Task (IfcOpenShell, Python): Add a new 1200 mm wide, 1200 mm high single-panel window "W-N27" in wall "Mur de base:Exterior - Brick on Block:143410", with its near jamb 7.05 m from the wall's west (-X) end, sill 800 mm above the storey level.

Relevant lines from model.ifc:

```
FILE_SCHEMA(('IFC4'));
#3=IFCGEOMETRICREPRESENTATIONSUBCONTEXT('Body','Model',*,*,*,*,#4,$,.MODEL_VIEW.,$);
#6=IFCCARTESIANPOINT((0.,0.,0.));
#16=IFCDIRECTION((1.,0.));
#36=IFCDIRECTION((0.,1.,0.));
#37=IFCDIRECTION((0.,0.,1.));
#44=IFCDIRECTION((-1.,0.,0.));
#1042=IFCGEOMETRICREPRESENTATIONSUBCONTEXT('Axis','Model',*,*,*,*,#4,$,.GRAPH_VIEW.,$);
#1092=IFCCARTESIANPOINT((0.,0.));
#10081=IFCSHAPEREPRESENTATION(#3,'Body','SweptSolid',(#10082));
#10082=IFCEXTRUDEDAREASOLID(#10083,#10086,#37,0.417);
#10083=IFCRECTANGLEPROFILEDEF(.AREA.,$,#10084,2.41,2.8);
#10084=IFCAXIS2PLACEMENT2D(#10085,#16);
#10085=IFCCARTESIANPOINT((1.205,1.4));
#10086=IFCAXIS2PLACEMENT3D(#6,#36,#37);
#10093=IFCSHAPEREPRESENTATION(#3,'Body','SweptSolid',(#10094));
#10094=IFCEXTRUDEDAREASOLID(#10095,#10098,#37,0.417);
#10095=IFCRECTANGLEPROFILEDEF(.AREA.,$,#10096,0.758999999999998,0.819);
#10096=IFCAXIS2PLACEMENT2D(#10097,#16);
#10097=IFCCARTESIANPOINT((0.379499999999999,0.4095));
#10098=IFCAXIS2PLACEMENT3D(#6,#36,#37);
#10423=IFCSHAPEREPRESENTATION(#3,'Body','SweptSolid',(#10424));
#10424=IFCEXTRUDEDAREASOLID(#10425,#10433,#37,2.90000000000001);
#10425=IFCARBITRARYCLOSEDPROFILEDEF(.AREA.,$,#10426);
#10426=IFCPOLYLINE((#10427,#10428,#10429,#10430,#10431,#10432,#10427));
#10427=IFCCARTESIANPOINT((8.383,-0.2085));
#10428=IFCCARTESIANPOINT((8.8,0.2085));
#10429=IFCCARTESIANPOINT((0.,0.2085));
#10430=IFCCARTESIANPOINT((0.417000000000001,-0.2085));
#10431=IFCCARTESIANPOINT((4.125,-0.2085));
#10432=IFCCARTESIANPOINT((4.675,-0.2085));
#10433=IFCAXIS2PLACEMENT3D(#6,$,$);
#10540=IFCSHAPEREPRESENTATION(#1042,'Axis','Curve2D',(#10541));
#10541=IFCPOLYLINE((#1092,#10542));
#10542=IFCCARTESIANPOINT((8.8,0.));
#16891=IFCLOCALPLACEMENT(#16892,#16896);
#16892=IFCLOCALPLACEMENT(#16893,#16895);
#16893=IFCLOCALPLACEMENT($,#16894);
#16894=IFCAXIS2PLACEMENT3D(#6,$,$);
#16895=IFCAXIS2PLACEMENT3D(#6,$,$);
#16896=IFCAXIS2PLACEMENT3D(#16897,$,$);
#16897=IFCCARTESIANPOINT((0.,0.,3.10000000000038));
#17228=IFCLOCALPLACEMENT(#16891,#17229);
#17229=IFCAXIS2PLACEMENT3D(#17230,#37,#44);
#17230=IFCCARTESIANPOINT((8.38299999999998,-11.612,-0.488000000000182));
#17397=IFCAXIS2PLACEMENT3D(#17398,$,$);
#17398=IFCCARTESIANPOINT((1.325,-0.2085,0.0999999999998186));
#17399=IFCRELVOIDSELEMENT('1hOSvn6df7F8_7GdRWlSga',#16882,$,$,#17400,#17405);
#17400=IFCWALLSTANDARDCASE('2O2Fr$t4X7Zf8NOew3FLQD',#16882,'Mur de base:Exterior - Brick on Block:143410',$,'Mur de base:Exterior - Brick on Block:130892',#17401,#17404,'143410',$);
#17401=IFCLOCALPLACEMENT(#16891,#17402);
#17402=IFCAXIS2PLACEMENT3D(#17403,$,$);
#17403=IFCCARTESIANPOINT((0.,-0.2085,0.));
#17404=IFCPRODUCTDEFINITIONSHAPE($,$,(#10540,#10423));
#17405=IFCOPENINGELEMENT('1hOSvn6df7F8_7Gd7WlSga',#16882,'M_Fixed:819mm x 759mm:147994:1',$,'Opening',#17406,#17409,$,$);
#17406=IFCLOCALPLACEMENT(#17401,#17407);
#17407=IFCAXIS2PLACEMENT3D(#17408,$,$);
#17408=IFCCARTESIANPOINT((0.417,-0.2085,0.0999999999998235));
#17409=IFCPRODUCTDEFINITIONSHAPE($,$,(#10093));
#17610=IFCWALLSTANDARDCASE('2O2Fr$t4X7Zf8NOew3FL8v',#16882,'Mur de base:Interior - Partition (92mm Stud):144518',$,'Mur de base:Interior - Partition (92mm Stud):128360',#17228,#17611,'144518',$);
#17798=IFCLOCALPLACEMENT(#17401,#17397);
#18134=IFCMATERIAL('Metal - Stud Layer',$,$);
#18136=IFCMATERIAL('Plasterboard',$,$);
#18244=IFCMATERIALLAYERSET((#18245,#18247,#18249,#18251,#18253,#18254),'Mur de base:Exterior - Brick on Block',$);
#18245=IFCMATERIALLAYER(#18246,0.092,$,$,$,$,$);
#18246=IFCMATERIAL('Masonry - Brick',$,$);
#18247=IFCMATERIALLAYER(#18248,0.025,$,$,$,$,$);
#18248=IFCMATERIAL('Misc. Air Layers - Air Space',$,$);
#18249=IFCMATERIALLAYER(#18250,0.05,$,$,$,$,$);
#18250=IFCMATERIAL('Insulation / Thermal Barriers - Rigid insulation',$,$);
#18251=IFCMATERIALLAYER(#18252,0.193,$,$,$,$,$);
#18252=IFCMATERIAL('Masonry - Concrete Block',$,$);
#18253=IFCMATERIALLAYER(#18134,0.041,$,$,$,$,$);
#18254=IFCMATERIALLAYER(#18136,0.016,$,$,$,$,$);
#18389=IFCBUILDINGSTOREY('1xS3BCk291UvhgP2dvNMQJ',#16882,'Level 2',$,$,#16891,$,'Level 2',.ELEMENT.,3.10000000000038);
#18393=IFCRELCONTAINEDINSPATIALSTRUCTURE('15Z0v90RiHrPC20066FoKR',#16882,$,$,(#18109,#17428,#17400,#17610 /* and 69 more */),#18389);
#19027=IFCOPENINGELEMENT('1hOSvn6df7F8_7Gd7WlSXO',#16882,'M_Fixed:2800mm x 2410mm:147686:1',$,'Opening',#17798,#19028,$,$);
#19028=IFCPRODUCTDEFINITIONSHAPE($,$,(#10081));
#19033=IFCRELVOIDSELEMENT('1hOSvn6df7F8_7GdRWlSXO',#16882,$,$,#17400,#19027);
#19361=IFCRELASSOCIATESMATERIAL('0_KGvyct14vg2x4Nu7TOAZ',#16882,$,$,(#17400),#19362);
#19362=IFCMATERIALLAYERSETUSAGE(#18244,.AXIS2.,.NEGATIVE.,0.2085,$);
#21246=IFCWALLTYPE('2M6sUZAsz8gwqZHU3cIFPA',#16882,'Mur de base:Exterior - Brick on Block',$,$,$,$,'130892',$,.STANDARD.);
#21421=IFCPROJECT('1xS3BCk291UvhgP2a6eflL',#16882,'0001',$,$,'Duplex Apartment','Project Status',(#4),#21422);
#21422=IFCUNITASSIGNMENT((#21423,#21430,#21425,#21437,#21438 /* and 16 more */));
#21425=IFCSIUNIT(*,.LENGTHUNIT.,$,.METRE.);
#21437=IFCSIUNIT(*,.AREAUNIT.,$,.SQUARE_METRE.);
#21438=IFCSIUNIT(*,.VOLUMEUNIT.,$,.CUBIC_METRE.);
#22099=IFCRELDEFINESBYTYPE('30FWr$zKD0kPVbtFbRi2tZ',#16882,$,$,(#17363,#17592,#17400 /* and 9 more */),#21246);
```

```python
import numpy as np
import ifcopenshell
import ifcopenshell.api.feature
import ifcopenshell.api.geometry
import ifcopenshell.api.root
import ifcopenshell.api.spatial
import ifcopenshell.geom
import ifcopenshell.util.element
import ifcopenshell.util.placement
import ifcopenshell.util.representation
import ifcopenshell.util.shape
import ifcopenshell.util.unit

model = ifcopenshell.open("model.ifc")
unit_scale = ifcopenshell.util.unit.calculate_unit_scale(model)
settings = ifcopenshell.geom.settings()


def volume(element):
    """Net volume in cubic metres, openings subtracted."""
    shape = ifcopenshell.geom.create_shape(settings, element)
    return ifcopenshell.util.shape.get_volume(shape.geometry)


wall = model.by_guid("2O2Fr$t4X7Zf8NOew3FLQD")
storey = ifcopenshell.util.element.get_container(wall, ifc_class="IfcBuildingStorey")
context = ifcopenshell.util.representation.get_context(model, "Model", "Body", "MODEL_VIEW")
before = volume(wall)

width, height, from_end, sill = 1.2, 1.2, 7.05, 0.8  # metres

# The wall runs along its own X axis, and the end named is its -X end.
wall_shape = ifcopenshell.geom.create_shape(settings, wall)
x, y, z = ifcopenshell.util.shape.get_vertices(wall_shape.geometry).T
start = x.min() + from_end
face, thickness = float(y.min()), float(y.max() - y.min())
wall_matrix = ifcopenshell.util.placement.get_local_placement(wall.ObjectPlacement)
level = ifcopenshell.util.placement.get_local_placement(storey.ObjectPlacement)[2, 3]


def in_wall(x, y):
    """Placement at x, y metres in the wall's axes, at sill height."""
    matrix = wall_matrix.copy()
    matrix[:, 3] = wall_matrix @ np.array([x / unit_scale, y / unit_scale, 0.0, 1.0])
    matrix[2, 3] = level + sill / unit_scale
    return matrix


# Opening: a box that overshoots both wall faces by 50 mm.
opening = ifcopenshell.api.root.create_entity(model, ifc_class="IfcOpeningElement", predefined_type="OPENING")
box = ifcopenshell.api.geometry.add_wall_representation(
    model, context=context, length=width, height=height, thickness=thickness + 0.1
)
ifcopenshell.api.geometry.assign_representation(model, product=opening, representation=box)
ifcopenshell.api.geometry.edit_object_placement(model, product=opening, matrix=in_wall(start, face - 0.05), is_si=False)
ifcopenshell.api.feature.add_feature(model, feature=opening, element=wall)

window = ifcopenshell.api.root.create_entity(model, ifc_class="IfcWindow", name="W-N27", predefined_type="WINDOW")
window.OverallWidth, window.OverallHeight = width / unit_scale, height / unit_scale
window.PartitioningType = "SINGLE_PANEL"
body = ifcopenshell.api.geometry.add_window_representation(
    model,
    context=context,
    overall_width=window.OverallWidth,
    overall_height=window.OverallHeight,
    partition_type="SINGLE_PANEL",
)
ifcopenshell.api.geometry.assign_representation(model, product=window, representation=body)
ifcopenshell.api.spatial.assign_container(model, products=[window], relating_structure=storey)
ifcopenshell.api.feature.add_filling(model, opening=opening, element=window)

# Centre the window in the wall's thickness.
ifcopenshell.api.geometry.edit_object_placement(model, product=window, matrix=in_wall(start, face), is_si=False)
window_shape = ifcopenshell.geom.create_shape(settings, window)
depth = ifcopenshell.util.shape.get_vertices(window_shape.geometry)[:, 1]
offset = face + thickness / 2 - (depth.min() + depth.max()) / 2
ifcopenshell.api.geometry.edit_object_placement(model, product=window, matrix=in_wall(start, offset), is_si=False)

after = volume(wall)

print(f"wall volume {before:.3f} -> {after:.3f} m3")

model.write("model_edited.ifc")
```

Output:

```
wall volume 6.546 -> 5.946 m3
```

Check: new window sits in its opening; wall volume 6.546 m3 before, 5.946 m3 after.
